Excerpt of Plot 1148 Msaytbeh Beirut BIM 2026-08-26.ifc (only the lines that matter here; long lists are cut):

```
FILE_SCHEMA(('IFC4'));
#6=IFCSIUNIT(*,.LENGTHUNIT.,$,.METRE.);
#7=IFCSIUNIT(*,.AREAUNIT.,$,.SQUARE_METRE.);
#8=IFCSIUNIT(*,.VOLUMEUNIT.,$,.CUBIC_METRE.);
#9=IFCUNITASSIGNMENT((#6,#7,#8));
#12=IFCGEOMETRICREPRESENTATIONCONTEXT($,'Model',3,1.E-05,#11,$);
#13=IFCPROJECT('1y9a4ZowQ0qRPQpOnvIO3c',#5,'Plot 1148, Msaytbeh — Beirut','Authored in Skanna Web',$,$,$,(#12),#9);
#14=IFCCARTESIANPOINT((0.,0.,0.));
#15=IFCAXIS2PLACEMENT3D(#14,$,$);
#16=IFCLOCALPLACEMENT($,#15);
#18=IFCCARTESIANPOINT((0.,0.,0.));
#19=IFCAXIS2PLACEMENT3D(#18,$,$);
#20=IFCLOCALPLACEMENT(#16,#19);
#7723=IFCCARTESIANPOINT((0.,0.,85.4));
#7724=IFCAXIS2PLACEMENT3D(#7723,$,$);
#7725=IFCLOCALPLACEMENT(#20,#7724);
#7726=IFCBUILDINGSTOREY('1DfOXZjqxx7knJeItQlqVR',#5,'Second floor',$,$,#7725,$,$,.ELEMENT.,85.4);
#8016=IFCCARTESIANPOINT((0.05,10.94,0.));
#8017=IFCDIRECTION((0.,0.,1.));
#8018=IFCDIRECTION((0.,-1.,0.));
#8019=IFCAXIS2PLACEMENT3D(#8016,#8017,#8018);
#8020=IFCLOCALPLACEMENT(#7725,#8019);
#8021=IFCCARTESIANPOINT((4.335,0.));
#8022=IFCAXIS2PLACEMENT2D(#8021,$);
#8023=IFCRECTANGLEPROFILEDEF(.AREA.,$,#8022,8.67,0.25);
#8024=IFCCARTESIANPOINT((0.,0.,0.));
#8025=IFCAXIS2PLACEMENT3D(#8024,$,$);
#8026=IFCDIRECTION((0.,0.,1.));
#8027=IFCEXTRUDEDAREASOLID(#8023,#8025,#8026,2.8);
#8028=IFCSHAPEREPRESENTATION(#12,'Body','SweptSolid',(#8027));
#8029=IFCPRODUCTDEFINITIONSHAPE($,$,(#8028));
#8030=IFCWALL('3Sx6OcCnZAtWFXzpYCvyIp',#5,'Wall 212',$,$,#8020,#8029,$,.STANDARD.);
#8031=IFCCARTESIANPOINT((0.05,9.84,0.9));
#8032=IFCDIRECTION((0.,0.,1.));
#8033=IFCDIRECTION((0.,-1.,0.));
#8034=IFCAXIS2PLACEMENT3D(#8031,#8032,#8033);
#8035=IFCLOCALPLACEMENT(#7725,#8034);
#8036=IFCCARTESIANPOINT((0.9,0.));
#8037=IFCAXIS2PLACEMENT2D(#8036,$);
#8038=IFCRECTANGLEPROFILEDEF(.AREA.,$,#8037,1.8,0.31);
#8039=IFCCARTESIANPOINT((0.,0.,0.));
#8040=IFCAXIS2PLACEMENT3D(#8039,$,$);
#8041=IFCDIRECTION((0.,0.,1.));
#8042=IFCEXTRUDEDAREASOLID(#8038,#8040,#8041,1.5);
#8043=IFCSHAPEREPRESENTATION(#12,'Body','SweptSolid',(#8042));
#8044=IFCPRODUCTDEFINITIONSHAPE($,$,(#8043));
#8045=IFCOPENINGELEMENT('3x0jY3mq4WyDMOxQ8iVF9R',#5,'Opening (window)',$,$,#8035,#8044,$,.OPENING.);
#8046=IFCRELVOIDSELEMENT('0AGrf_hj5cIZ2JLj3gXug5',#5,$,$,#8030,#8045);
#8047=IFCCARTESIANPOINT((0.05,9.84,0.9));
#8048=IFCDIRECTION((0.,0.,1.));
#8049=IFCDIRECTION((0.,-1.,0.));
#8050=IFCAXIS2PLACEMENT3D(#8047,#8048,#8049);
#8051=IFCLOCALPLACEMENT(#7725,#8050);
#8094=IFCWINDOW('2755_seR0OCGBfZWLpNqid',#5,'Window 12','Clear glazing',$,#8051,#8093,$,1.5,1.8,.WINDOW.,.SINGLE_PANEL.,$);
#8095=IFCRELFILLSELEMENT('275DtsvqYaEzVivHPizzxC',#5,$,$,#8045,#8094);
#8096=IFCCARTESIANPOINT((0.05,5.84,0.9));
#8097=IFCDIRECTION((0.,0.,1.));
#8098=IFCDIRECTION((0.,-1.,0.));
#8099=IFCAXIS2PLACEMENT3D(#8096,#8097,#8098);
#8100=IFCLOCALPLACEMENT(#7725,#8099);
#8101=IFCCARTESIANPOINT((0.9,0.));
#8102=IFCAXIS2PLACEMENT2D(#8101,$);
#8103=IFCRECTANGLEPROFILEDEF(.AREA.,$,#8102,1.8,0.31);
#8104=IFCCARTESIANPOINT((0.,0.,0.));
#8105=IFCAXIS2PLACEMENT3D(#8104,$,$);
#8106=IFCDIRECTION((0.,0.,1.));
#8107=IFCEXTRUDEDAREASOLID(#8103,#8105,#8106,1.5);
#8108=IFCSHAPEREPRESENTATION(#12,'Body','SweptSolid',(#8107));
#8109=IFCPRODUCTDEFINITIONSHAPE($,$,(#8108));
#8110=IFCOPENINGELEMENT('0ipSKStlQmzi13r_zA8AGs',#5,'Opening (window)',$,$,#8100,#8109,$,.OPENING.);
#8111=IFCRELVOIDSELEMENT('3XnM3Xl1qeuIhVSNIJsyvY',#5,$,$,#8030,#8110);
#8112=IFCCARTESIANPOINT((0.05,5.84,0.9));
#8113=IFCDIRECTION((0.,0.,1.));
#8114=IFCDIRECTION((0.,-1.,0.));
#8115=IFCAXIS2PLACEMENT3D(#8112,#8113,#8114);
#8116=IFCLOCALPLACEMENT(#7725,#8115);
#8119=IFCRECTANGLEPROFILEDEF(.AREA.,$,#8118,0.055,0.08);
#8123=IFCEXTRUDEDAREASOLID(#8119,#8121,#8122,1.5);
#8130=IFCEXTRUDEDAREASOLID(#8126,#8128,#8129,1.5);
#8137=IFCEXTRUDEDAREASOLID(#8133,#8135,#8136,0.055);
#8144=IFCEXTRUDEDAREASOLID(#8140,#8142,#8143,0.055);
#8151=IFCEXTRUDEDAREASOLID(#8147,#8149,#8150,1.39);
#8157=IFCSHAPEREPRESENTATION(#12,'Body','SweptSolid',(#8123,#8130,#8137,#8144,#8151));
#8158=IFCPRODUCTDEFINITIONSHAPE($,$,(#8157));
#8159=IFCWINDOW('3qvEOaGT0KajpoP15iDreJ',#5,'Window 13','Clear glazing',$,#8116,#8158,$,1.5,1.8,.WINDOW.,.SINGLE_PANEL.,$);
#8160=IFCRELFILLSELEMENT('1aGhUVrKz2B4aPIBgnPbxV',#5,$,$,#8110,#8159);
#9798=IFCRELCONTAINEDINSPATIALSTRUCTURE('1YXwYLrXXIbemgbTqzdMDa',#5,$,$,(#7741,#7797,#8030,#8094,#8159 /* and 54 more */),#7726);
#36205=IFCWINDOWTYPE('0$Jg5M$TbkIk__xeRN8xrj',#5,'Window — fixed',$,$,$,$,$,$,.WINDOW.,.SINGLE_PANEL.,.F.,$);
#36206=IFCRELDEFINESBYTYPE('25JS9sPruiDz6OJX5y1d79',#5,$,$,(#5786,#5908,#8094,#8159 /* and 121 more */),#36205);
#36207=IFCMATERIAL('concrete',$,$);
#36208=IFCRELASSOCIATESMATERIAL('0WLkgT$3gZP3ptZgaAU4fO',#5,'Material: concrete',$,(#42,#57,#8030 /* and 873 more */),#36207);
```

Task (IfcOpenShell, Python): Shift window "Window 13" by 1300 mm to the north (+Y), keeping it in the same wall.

```python
import ifcopenshell
import ifcopenshell.api.geometry
import ifcopenshell.util.placement
import ifcopenshell.util.unit

model = ifcopenshell.open("Plot 1148 Msaytbeh Beirut BIM 2026-08-26.ifc")
unit_scale = ifcopenshell.util.unit.calculate_unit_scale(model)

window = model.by_guid("3qvEOaGT0KajpoP15iDreJ")
opening = window.FillsVoids[0].RelatingOpeningElement
wall = opening.VoidsElements[0].RelatingBuildingElement

wall_matrix = ifcopenshell.util.placement.get_local_placement(wall.ObjectPlacement)
shift = wall_matrix[:3, 0] * -1.3 / unit_scale
before = ifcopenshell.util.placement.get_local_placement(window.ObjectPlacement)[:3, 3].copy()

# The window is not placed relative to its opening, so move both.
for product in (opening, window):
    matrix = ifcopenshell.util.placement.get_local_placement(product.ObjectPlacement)
    matrix[:3, 3] += shift
    ifcopenshell.api.geometry.edit_object_placement(model, product=product, matrix=matrix, is_si=False)

after = ifcopenshell.util.placement.get_local_placement(window.ObjectPlacement)[:3, 3]
print("window moved by", (after - before).round(3) + 0.0)

model.write("Plot 1148 Msaytbeh Beirut BIM 2026-08-26-out.ifc")
```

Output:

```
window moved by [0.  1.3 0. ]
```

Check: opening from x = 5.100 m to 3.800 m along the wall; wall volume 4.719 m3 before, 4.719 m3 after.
